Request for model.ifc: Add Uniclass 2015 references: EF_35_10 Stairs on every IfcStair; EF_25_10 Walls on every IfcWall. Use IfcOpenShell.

First a look at what the model holds.

```python
import ifcopenshell

model = ifcopenshell.open("model.ifc")
print(model.schema)
print("classifications:", [c.Name for c in model.by_type("IfcClassification")])
for ifc_class in ("IfcDoor", "IfcRoof", "IfcStair", "IfcWall", "IfcWindow"):
    print(ifc_class, len(model.by_type(ifc_class)))
```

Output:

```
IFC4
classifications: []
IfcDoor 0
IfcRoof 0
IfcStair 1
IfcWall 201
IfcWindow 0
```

```python
import ifcopenshell
import ifcopenshell.api.classification

model = ifcopenshell.open("model.ifc")

system = ifcopenshell.api.classification.add_classification(model, classification="Uniclass 2015")

codes = {
    "IfcStair": ("EF_35_10", "Stairs"),
    "IfcWall": ("EF_25_10", "Walls"),
}
for ifc_class, (code, name) in codes.items():
    products = model.by_type(ifc_class)
    ifcopenshell.api.classification.add_reference(
        model, products=products, classification=system, identification=code, name=name
    )
    print(code, len(products))

model.write("model_edited.ifc")
```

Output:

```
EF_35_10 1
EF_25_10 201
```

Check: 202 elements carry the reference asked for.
